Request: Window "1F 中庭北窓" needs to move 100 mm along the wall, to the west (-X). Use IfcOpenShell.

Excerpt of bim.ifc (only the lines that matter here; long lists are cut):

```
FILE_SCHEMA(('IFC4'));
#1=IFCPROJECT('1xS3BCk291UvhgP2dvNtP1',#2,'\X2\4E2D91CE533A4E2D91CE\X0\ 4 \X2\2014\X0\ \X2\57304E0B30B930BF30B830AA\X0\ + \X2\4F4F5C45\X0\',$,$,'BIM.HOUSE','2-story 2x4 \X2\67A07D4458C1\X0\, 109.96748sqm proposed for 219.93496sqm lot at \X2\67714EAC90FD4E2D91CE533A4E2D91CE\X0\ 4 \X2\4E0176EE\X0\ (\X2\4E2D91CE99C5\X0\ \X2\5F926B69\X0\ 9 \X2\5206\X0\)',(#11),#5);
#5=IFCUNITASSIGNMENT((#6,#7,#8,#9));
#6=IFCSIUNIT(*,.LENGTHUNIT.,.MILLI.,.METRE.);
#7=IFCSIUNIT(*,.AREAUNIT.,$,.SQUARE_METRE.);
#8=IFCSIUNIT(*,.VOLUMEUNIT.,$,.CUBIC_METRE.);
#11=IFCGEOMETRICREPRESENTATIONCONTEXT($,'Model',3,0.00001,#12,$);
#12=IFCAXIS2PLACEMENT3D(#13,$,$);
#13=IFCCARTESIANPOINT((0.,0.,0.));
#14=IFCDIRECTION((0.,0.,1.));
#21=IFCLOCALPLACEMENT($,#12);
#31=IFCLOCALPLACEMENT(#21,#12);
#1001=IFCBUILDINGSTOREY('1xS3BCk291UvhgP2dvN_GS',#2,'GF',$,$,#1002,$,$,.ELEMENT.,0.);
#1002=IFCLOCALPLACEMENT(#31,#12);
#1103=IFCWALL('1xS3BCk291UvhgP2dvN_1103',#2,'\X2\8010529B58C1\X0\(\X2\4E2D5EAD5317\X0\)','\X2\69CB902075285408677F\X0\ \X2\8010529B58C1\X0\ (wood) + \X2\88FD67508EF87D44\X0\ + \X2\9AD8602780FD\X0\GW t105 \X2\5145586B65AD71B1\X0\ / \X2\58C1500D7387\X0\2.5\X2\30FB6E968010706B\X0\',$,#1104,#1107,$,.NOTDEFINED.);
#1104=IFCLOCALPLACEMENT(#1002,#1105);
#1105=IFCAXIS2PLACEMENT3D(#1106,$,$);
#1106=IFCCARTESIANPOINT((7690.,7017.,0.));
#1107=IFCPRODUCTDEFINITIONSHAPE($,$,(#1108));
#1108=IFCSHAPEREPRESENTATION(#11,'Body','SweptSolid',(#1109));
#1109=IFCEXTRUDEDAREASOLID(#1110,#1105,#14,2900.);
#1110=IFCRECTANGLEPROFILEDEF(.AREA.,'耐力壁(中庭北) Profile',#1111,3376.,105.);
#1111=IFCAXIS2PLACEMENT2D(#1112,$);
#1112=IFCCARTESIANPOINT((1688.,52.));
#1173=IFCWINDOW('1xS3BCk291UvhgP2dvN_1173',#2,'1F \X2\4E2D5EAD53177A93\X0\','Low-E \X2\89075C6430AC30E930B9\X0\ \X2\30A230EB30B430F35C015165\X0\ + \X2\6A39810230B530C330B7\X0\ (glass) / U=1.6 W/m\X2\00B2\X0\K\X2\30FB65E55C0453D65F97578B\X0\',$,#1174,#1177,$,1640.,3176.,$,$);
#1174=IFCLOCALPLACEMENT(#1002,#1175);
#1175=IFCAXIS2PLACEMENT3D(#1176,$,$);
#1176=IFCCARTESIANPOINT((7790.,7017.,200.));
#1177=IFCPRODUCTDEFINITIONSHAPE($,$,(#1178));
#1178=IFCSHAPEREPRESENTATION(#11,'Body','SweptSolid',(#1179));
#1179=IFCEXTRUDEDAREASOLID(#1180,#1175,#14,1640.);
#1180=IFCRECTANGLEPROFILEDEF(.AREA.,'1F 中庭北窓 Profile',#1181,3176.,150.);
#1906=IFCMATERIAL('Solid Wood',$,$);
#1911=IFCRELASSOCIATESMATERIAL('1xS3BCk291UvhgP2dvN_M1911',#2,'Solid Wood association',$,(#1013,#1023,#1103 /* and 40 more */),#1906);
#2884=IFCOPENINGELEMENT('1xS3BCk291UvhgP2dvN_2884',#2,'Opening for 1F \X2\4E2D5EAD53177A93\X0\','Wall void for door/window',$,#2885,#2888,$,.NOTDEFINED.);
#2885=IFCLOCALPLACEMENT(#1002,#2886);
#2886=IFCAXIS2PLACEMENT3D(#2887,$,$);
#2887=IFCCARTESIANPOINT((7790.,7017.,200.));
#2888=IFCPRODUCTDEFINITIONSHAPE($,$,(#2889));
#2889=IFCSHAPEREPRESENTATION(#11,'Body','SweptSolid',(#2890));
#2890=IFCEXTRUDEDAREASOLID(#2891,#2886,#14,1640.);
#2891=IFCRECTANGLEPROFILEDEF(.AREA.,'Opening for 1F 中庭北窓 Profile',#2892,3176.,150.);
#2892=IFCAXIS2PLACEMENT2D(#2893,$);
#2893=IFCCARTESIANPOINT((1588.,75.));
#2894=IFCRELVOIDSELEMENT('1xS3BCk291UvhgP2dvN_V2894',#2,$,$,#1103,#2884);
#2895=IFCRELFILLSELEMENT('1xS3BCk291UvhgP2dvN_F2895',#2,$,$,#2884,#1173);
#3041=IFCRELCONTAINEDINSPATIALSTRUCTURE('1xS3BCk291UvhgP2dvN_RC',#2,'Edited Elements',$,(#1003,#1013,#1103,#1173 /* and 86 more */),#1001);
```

```python
import ifcopenshell
import ifcopenshell.api.geometry
import ifcopenshell.util.placement

model = ifcopenshell.open("bim.ifc")

window = model.by_id(1173)
opening = window.FillsVoids[0].RelatingOpeningElement
wall = opening.VoidsElements[0].RelatingBuildingElement

wall_matrix = ifcopenshell.util.placement.get_local_placement(wall.ObjectPlacement)
shift = wall_matrix[:3, 0] * -100.0
before = ifcopenshell.util.placement.get_local_placement(window.ObjectPlacement)[:3, 3].copy()

# The window is not placed relative to its opening, so move both.
for product in (opening, window):
    matrix = ifcopenshell.util.placement.get_local_placement(product.ObjectPlacement)
    matrix[:3, 3] += shift
    ifcopenshell.api.geometry.edit_object_placement(model, product=product, matrix=matrix, is_si=False)

after = ifcopenshell.util.placement.get_local_placement(window.ObjectPlacement)[:3, 3]
print("window moved by", (after - before).round(3) + 0.0)

model.write("bim_updated.ifc")
```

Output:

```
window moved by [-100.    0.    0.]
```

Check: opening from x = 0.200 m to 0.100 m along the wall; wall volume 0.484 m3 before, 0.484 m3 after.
